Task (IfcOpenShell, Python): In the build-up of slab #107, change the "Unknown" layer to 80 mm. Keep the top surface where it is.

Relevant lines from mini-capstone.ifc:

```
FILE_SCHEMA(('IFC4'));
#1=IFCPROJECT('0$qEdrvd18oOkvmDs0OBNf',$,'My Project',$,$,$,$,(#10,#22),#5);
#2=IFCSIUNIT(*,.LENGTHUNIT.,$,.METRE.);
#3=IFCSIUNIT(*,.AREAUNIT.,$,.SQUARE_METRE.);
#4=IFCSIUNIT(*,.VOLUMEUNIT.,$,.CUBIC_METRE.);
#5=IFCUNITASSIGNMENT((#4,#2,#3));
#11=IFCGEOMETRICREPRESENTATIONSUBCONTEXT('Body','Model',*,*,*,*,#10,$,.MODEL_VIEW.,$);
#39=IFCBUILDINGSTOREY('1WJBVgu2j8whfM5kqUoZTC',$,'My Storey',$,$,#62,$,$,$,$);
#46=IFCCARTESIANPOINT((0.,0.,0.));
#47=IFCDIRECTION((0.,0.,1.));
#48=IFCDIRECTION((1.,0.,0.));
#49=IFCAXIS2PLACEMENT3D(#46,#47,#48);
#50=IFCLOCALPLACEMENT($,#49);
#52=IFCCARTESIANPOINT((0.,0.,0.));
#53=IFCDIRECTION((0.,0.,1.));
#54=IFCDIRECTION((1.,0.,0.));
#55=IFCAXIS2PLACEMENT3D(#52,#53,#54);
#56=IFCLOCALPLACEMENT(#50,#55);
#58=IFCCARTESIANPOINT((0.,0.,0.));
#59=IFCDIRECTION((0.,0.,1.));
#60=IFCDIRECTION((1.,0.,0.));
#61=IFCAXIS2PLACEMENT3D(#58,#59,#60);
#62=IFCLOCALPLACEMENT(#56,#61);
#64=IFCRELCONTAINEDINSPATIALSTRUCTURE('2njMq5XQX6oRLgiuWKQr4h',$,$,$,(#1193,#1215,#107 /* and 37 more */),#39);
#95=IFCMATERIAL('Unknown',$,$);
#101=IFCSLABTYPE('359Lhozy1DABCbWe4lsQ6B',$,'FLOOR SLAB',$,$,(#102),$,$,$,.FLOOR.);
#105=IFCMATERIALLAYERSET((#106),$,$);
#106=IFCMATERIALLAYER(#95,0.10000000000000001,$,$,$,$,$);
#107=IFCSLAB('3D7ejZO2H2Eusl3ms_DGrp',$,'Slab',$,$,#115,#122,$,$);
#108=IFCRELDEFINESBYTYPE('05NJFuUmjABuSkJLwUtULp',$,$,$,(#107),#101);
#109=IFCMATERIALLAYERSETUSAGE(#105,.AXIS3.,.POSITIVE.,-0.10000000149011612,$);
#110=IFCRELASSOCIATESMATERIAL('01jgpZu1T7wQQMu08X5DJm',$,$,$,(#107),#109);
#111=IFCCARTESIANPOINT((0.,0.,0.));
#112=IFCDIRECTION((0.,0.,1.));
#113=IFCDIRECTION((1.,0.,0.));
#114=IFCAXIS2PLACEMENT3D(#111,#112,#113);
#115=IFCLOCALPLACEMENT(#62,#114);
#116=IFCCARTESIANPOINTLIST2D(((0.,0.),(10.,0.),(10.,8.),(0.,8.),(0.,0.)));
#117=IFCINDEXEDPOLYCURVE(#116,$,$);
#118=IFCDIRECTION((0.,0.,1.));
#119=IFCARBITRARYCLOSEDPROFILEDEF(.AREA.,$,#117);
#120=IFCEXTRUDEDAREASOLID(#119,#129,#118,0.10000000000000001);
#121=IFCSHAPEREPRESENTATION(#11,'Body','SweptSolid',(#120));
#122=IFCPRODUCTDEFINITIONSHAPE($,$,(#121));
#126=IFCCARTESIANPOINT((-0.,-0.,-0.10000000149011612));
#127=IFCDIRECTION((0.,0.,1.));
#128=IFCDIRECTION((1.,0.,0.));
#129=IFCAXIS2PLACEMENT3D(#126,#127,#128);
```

```python
import ifcopenshell
import ifcopenshell.util.element
import ifcopenshell.util.representation
import ifcopenshell.util.unit

model = ifcopenshell.open("mini-capstone.ifc")
unit_scale = ifcopenshell.util.unit.calculate_unit_scale(model)

layer_set = model.by_id(105)
layer = next(l for l in layer_set.MaterialLayers if l.Material and l.Material.Name == "Unknown")
change = 0.08 / unit_scale - layer.LayerThickness
layer.LayerThickness += change

# Geometry does not follow the layer set by itself.
slabs = [e for e in ifcopenshell.util.element.get_elements_by_material(model, layer_set) if e.is_a("IfcSlab")]
for slab in sorted(slabs, key=lambda e: e.id()):
    body = ifcopenshell.util.representation.get_representation(slab, "Model", "Body")
    solid = body.Items[0]
    old_depth = solid.Depth
    solid.Depth += change
    # Extruded upwards: lower the start of the extrusion so the top stays.
    x, y, z = solid.Position.Location.Coordinates
    solid.Position.Location = model.createIfcCartesianPoint((x, y, z - change))
    print(slab.id(), f"{old_depth:g} -> {solid.Depth:g}")

# The layers are counted up from the underside, which has moved.
for usage in {ifcopenshell.util.element.get_material(slab) for slab in slabs}:
    usage.OffsetFromReferenceLine -= change

model.write("mini-capstone_rev.ifc")
```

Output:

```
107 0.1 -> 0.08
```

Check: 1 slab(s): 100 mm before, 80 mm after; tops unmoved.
